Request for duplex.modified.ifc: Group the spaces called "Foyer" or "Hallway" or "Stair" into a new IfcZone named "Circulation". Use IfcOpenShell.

First a look at what the model holds.

```python
import ifcopenshell

model = ifcopenshell.open("duplex.modified.ifc")
print(model.schema)
seen = {}
for space in model.by_type("IfcSpace"):
    seen[space.LongName] = seen.get(space.LongName, 0) + 1
for name, count in sorted(seen.items(), key=str):
    print(count, "x", name)
print("zones:", [z.Name for z in model.by_type("IfcZone")][:20])
```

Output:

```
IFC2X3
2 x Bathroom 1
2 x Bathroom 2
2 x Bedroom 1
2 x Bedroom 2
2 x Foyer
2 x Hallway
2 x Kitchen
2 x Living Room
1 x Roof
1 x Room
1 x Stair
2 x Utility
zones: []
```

```python
import ifcopenshell
import ifcopenshell.api.group
import ifcopenshell.api.root

model = ifcopenshell.open("duplex.modified.ifc")

names = {"Foyer", "Hallway", "Stair"}
spaces = [s for s in model.by_type("IfcSpace") if s.LongName in names]

zone = ifcopenshell.api.root.create_entity(model, ifc_class="IfcZone", name="Circulation")
ifcopenshell.api.group.assign_group(model, products=spaces, group=zone)
print(len(spaces), "spaces in", zone.Name)

model.write("duplex.modified_updated.ifc")
```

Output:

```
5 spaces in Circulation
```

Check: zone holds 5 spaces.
